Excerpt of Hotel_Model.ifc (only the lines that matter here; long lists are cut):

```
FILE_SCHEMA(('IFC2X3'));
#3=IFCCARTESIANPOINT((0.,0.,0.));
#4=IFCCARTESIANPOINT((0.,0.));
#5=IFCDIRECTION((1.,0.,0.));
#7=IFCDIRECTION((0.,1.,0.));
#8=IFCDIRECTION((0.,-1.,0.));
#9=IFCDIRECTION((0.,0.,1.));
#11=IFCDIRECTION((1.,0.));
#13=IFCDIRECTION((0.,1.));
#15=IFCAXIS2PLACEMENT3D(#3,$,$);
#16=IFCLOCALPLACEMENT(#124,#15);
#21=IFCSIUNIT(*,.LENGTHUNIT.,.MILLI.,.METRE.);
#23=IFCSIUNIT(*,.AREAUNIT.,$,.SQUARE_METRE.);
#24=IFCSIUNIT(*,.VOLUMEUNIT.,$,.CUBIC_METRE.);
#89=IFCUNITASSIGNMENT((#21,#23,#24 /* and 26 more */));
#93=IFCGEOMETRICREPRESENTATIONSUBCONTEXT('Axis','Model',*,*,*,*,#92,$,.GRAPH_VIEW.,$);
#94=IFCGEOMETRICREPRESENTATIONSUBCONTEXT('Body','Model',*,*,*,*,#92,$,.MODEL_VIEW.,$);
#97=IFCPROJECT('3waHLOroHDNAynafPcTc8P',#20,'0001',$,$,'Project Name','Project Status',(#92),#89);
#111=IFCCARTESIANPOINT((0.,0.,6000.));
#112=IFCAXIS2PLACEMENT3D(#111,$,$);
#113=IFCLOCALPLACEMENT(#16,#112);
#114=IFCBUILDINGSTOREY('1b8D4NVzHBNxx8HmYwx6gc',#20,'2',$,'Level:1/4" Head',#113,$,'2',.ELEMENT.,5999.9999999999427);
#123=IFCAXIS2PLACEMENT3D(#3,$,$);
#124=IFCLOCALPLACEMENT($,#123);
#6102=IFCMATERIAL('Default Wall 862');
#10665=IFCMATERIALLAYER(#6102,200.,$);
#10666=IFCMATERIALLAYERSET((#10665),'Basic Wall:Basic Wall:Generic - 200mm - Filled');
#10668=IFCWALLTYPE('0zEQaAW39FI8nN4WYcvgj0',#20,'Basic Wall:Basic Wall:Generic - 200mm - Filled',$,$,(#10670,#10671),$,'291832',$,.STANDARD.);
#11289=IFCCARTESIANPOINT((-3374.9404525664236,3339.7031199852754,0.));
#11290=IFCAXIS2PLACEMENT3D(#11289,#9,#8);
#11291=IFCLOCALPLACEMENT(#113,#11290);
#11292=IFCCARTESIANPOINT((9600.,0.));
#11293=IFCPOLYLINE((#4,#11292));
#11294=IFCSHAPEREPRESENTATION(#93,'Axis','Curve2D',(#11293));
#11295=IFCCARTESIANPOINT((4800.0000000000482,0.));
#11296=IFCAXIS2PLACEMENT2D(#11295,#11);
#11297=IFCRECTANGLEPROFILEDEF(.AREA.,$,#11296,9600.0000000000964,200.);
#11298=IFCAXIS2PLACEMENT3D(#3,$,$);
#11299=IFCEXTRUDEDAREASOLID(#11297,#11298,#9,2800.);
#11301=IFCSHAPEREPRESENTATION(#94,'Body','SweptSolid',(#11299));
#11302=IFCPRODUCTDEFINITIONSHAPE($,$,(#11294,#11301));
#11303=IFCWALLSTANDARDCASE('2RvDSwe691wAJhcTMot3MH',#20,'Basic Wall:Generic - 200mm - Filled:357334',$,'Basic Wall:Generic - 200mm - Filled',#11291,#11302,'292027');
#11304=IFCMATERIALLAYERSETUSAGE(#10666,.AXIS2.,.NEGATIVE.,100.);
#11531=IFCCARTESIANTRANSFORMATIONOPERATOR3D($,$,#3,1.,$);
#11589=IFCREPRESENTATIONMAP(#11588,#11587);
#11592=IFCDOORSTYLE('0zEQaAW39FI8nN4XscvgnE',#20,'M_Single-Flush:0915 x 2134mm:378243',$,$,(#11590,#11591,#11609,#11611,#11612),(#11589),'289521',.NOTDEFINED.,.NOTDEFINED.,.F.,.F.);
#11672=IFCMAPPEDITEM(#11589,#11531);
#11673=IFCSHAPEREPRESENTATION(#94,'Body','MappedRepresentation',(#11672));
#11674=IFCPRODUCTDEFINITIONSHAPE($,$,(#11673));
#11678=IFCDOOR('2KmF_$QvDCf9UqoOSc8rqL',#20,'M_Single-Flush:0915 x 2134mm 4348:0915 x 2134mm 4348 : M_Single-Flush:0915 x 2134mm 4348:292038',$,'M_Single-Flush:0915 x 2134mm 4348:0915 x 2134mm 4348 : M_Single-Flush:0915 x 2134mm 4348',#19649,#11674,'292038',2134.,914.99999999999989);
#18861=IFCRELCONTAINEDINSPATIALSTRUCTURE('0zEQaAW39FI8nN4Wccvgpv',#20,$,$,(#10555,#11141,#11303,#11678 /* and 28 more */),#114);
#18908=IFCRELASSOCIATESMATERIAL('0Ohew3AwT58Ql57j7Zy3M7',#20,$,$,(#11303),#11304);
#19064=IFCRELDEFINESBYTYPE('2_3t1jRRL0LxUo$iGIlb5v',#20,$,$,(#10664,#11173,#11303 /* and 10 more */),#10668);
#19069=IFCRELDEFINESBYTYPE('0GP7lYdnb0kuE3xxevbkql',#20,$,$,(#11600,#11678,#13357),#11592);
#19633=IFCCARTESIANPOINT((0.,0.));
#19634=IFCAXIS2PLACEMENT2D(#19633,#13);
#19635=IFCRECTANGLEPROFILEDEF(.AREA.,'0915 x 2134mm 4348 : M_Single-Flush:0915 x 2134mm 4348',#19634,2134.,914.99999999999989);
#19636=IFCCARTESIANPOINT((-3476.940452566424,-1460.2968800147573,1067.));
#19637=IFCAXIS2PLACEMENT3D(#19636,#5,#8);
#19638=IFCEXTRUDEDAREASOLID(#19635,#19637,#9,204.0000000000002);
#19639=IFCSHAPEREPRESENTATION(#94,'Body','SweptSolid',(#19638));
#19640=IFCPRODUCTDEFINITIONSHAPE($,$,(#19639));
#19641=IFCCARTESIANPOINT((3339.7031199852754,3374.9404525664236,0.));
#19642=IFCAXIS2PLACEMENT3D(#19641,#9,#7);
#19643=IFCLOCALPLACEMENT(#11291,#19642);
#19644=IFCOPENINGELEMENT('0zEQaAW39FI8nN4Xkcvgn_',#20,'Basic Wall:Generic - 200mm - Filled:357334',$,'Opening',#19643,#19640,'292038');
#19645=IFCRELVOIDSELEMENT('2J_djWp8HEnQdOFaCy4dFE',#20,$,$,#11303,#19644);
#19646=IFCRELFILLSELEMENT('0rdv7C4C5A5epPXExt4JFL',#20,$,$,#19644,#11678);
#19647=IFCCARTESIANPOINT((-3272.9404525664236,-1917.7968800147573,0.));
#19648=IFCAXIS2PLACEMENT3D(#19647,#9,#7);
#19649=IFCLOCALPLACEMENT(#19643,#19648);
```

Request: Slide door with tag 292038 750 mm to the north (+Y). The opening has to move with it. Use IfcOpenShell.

```python
import ifcopenshell
import ifcopenshell.api.geometry
import ifcopenshell.util.placement

model = ifcopenshell.open("Hotel_Model.ifc")

door = model.by_guid("2KmF_$QvDCf9UqoOSc8rqL")
opening = door.FillsVoids[0].RelatingOpeningElement
wall = opening.VoidsElements[0].RelatingBuildingElement

wall_matrix = ifcopenshell.util.placement.get_local_placement(wall.ObjectPlacement)
shift = wall_matrix[:3, 0] * -750.0
before = ifcopenshell.util.placement.get_local_placement(door.ObjectPlacement)[:3, 3].copy()

# The door is placed relative to its opening, so it follows when the opening moves.
matrix = ifcopenshell.util.placement.get_local_placement(opening.ObjectPlacement)
matrix[:3, 3] += shift
ifcopenshell.api.geometry.edit_object_placement(
    model, product=opening, matrix=matrix, is_si=False, should_transform_children=True
)

after = ifcopenshell.util.placement.get_local_placement(door.ObjectPlacement)[:3, 3]
print("door moved by", (after - before).round(3) + 0.0)

model.write("Hotel_Model-out.ifc")
```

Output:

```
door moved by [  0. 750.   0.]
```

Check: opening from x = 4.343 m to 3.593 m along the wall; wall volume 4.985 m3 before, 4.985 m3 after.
